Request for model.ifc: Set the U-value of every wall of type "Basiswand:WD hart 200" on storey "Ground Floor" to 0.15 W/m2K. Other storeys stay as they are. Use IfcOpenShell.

First a look at what the model holds.

```python
import ifcopenshell
import ifcopenshell.util.element

model = ifcopenshell.open("model.ifc")
print(model.schema)
storey = next(s for s in model.by_type("IfcBuildingStorey") if s.Name == "Ground Floor")
walls = [e for e in ifcopenshell.util.element.get_decomposition(storey) if e.is_a("IfcWall")]
seen = {}
for e in walls:
    element_type = ifcopenshell.util.element.get_type(e)
    key = (element_type.Name if element_type != e and element_type else None, ifcopenshell.util.element.get_pset(e, "Pset_WallCommon", "ThermalTransmittance"))
    seen[key] = seen.get(key, 0) + 1
for (name, value), count in sorted(seen.items(), key=str):
    print(count, "x", name, "|", value)
```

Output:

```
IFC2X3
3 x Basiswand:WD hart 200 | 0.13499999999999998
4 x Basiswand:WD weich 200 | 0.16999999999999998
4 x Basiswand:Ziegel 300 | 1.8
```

```python
import ifcopenshell
import ifcopenshell.api.pset
import ifcopenshell.util.element

model = ifcopenshell.open("model.ifc")

storey = next(s for s in model.by_type("IfcBuildingStorey") if s.Name == "Ground Floor")
walls = [e for e in ifcopenshell.util.element.get_decomposition(storey) if e.is_a("IfcWall")]

count = 0
for e in walls:
    element_type = ifcopenshell.util.element.get_type(e)
    if element_type in (None, e) or element_type.Name != "Basiswand:WD hart 200":
        continue
    # add_pset returns the element's existing set when there is one.
    pset = ifcopenshell.api.pset.add_pset(model, product=e, name="Pset_WallCommon")
    ifcopenshell.api.pset.edit_pset(model, pset=pset, properties={"ThermalTransmittance": 0.15})
    count += 1

print(count, "walls updated")

model.write("model_rev.ifc")
```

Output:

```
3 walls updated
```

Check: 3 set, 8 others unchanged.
